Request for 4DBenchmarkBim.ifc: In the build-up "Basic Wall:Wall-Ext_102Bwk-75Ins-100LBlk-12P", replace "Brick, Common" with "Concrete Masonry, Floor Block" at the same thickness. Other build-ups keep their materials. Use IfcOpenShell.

First a look at what the model holds.

```python
import ifcopenshell
import ifcopenshell.util.element

model = ifcopenshell.open("4DBenchmarkBim.ifc")
print(model.schema)
for layer_set in model.by_type("IfcMaterialLayerSet"):
    if layer_set.LayerSetName == "Basic Wall:Wall-Ext_102Bwk-75Ins-100LBlk-12P":
        for layer in layer_set.MaterialLayers:
            print(layer.id(), layer.Material and layer.Material.Name, layer.LayerThickness, sep=" | ")
        print(len(ifcopenshell.util.element.get_elements_by_material(model, layer_set)), "elements and types use it")
print(sorted(m.Name for m in model.by_type("IfcMaterial") if m.Name)[:60])
```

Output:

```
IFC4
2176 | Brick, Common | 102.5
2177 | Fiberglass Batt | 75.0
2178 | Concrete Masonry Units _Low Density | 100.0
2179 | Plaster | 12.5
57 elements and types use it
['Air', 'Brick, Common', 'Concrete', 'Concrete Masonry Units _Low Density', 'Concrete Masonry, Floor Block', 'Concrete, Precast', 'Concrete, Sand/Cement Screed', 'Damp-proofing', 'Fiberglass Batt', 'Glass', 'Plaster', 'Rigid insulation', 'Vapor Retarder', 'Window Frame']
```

```python
import ifcopenshell
import ifcopenshell.api.material

model = ifcopenshell.open("4DBenchmarkBim.ifc")

layer_set = next(s for s in model.by_type("IfcMaterialLayerSet") if s.LayerSetName == "Basic Wall:Wall-Ext_102Bwk-75Ins-100LBlk-12P")
layer = next(l for l in layer_set.MaterialLayers if l.Material and l.Material.Name == "Brick, Common")
material = next(m for m in model.by_type("IfcMaterial") if m.Name == "Concrete Masonry, Floor Block")

# Point this one layer at the other material; renaming the old one would change it everywhere.
ifcopenshell.api.material.edit_layer(model, layer=layer, attributes={"Name": material.Name}, material=material)

print([l.Material.Name if l.Material else None for l in layer_set.MaterialLayers])

model.write("4DBenchmarkBim_edited.ifc")
```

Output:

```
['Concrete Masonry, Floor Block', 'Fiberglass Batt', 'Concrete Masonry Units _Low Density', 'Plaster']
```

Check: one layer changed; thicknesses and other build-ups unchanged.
